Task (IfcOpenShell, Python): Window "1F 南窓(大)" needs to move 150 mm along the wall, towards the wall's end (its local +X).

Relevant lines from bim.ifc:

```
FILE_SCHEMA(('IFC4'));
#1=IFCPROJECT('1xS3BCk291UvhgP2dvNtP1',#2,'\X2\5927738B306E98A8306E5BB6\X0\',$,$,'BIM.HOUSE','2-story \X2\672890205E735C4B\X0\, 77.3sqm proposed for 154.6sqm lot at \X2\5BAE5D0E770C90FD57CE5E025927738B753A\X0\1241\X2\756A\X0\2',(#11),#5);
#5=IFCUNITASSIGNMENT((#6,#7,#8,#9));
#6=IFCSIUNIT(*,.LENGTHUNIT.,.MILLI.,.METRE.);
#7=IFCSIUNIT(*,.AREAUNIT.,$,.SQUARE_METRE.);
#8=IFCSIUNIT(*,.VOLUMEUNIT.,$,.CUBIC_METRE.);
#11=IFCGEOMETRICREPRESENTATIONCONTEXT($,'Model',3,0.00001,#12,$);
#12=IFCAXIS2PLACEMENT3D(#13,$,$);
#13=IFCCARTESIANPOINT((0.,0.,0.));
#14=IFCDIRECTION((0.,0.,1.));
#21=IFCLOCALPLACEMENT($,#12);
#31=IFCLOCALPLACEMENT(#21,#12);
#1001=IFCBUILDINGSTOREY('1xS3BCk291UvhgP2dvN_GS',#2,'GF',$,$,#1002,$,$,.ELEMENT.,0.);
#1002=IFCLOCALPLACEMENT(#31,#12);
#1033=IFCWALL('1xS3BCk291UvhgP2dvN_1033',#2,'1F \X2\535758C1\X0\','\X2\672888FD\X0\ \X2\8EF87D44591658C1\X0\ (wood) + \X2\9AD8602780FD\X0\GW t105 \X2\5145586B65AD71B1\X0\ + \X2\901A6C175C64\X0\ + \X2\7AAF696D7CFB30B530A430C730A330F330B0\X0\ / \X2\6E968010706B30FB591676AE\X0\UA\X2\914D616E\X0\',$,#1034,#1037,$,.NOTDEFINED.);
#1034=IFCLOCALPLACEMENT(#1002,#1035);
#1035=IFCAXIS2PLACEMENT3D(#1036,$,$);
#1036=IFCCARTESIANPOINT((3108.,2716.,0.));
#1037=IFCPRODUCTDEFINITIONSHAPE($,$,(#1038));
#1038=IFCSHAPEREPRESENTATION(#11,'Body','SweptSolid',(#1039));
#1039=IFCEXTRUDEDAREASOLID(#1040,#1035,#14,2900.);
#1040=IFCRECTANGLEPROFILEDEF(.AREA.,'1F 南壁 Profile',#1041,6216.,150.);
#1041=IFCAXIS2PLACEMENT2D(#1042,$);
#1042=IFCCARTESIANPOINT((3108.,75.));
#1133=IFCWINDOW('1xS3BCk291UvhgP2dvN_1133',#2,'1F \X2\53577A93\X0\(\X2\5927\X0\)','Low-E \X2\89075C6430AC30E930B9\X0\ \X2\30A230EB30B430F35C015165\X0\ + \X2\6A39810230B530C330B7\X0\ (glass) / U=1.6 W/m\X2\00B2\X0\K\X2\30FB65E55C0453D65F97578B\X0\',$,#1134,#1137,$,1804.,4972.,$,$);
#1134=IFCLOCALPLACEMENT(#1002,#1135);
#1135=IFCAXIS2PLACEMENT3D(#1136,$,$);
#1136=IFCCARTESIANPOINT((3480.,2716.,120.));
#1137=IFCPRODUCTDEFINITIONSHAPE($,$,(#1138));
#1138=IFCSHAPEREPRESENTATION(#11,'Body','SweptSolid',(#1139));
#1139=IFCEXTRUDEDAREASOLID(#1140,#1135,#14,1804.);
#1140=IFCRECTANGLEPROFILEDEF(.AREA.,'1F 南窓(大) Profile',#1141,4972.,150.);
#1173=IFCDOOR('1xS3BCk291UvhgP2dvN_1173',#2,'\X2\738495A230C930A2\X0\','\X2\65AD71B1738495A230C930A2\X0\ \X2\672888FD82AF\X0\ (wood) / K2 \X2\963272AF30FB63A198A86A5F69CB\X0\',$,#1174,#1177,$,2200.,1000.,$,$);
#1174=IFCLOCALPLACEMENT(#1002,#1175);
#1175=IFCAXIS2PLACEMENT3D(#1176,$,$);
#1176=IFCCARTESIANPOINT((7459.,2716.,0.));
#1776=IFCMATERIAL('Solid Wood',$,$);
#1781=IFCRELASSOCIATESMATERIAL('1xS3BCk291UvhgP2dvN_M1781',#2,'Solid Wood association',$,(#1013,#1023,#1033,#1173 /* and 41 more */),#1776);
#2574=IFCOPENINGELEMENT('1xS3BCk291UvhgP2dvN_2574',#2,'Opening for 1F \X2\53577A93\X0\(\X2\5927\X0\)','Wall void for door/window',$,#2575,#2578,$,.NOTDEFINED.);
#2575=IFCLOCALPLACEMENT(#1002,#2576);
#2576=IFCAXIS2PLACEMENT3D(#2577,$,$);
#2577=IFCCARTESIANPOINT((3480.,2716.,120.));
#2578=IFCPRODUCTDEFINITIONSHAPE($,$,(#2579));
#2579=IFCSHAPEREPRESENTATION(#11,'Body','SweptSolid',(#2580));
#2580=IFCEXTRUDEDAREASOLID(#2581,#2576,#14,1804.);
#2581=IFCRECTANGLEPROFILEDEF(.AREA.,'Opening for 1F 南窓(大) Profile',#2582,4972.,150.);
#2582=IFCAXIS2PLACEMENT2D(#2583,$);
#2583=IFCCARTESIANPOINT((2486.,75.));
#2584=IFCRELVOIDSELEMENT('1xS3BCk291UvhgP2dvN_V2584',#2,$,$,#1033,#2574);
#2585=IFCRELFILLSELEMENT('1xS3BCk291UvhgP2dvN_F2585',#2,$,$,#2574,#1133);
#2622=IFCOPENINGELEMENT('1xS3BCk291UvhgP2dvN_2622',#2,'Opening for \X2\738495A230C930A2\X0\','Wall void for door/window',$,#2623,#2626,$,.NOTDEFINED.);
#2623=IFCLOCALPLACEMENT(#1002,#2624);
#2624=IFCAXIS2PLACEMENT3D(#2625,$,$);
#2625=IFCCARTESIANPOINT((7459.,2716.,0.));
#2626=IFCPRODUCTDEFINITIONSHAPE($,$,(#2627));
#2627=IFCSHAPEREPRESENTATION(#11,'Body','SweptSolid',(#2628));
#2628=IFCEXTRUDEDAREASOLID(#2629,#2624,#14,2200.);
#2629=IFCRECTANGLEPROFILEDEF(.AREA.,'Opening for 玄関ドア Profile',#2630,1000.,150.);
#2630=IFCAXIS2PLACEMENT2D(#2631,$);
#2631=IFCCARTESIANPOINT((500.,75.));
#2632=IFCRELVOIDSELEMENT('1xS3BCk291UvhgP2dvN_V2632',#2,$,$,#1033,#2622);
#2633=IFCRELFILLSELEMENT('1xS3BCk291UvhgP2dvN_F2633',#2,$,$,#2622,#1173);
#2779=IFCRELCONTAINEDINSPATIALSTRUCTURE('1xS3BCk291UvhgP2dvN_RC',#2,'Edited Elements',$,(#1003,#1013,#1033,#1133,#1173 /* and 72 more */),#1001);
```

```python
import ifcopenshell
import ifcopenshell.api.geometry
import ifcopenshell.util.placement

model = ifcopenshell.open("bim.ifc")

window = model.by_guid("1xS3BCk291UvhgP2dvN_1133")
opening = window.FillsVoids[0].RelatingOpeningElement
wall = opening.VoidsElements[0].RelatingBuildingElement

wall_matrix = ifcopenshell.util.placement.get_local_placement(wall.ObjectPlacement)
shift = wall_matrix[:3, 0] * 150.0
before = ifcopenshell.util.placement.get_local_placement(window.ObjectPlacement)[:3, 3].copy()

# The window is not placed relative to its opening, so move both.
for product in (opening, window):
    matrix = ifcopenshell.util.placement.get_local_placement(product.ObjectPlacement)
    matrix[:3, 3] += shift
    ifcopenshell.api.geometry.edit_object_placement(model, product=product, matrix=matrix, is_si=False)

after = ifcopenshell.util.placement.get_local_placement(window.ObjectPlacement)[:3, 3]
print("window moved by", (after - before).round(3) + 0.0)

model.write("bim_updated.ifc")
```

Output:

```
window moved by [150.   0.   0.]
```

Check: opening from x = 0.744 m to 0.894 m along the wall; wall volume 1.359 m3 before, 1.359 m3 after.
